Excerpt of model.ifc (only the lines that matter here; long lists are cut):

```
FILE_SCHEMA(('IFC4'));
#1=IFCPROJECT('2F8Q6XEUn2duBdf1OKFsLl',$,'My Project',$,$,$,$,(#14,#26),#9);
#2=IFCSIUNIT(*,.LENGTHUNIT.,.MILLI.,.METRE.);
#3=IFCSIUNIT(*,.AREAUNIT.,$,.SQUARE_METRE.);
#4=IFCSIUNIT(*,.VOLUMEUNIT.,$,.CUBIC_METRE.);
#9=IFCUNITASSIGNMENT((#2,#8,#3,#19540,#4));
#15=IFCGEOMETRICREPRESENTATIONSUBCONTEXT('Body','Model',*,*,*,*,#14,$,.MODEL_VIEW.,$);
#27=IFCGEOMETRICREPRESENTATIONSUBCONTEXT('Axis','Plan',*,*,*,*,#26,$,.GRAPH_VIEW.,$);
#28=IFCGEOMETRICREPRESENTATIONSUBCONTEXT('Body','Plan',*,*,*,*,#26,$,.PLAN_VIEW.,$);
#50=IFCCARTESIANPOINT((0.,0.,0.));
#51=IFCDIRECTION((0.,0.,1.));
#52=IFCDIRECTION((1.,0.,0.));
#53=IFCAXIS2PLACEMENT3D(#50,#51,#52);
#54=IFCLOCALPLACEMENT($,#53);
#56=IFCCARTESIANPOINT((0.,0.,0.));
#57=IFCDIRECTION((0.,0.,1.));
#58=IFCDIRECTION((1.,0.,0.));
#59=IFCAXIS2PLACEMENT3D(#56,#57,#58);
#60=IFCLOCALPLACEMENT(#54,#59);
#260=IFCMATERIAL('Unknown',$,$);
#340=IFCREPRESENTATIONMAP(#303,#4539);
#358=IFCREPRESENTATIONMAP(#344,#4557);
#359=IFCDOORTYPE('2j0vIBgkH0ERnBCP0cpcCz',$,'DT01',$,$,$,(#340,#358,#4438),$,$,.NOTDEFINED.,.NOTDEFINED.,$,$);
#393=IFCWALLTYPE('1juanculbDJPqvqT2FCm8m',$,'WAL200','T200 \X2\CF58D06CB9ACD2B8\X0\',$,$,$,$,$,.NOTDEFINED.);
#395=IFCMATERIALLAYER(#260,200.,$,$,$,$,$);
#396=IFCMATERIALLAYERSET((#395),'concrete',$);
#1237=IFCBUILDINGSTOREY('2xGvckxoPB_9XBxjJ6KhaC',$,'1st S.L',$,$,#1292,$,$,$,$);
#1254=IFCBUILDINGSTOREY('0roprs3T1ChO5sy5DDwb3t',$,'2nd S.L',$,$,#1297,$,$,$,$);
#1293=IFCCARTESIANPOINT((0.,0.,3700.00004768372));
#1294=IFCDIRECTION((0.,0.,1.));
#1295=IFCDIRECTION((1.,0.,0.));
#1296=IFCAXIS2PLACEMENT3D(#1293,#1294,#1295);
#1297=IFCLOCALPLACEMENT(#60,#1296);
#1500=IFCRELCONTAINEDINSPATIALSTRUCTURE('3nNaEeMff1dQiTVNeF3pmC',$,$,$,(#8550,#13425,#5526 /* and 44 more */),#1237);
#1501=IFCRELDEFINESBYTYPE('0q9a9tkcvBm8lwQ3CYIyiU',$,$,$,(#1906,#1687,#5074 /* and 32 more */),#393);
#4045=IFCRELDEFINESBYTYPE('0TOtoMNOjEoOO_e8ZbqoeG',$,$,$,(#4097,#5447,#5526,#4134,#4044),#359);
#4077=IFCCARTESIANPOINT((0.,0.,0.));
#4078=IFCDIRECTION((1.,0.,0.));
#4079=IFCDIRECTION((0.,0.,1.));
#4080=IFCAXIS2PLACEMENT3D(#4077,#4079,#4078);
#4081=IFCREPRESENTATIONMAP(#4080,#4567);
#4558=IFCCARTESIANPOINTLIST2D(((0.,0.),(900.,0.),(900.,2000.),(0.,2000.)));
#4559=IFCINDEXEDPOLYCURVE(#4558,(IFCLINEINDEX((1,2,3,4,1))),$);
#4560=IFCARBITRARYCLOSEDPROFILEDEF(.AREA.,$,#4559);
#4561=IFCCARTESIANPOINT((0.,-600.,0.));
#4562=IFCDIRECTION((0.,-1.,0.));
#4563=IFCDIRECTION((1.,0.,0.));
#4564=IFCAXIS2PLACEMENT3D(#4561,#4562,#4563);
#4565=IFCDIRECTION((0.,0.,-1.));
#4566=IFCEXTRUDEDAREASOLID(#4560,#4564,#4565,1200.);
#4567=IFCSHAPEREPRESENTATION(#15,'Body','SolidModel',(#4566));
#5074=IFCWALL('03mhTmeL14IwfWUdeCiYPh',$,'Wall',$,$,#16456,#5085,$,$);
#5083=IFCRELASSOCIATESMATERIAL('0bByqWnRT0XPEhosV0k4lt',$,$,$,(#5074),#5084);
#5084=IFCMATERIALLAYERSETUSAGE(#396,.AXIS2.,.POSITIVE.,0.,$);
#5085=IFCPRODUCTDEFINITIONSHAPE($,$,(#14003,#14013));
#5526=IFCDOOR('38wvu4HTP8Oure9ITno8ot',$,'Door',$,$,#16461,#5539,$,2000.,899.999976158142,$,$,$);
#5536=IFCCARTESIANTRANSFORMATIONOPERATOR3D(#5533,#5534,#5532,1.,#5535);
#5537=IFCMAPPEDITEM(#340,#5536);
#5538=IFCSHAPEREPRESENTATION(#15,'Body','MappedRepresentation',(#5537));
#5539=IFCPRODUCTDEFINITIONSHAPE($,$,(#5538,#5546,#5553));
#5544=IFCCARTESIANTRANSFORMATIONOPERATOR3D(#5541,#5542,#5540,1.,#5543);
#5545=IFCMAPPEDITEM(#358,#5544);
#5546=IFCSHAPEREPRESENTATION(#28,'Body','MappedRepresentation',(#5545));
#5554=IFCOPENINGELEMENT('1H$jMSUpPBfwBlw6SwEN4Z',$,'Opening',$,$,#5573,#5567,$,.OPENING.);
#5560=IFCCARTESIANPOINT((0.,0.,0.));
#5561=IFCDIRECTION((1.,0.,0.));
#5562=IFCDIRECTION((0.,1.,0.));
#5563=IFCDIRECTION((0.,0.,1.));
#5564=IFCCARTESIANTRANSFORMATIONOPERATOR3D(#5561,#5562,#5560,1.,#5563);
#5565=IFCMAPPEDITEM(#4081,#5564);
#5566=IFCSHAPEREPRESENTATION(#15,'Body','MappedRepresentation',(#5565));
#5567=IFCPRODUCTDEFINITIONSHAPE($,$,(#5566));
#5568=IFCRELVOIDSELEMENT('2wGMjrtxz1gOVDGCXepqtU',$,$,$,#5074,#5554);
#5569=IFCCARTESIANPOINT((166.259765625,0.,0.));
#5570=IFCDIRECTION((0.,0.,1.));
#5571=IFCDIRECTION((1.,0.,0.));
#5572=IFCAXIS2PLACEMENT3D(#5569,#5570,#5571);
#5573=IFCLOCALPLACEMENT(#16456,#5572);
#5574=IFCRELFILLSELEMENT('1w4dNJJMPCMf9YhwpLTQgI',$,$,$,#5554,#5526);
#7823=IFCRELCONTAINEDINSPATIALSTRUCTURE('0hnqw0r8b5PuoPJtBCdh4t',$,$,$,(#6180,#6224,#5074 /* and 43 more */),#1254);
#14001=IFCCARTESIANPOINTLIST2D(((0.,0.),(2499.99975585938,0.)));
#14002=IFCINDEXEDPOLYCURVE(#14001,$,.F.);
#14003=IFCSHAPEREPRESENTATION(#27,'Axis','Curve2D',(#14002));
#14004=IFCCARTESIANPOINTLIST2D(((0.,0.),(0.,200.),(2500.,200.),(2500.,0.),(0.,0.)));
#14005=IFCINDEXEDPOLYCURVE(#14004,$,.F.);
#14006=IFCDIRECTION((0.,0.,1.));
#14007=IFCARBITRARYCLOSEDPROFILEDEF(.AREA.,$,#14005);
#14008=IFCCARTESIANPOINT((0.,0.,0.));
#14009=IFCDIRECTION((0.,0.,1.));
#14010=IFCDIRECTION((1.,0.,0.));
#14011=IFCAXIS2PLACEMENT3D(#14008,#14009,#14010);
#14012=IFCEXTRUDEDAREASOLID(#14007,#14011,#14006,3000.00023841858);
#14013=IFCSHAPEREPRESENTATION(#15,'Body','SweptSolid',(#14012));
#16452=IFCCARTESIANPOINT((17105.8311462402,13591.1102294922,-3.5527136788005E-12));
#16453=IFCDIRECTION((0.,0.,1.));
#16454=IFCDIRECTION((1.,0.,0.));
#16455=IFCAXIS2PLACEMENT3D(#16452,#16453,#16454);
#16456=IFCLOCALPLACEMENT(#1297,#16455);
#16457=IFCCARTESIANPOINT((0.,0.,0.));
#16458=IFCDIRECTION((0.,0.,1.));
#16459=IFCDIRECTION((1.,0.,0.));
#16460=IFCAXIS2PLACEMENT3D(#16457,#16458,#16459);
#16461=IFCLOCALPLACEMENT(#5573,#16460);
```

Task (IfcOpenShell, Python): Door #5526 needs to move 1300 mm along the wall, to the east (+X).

```python
import ifcopenshell
import ifcopenshell.api.geometry
import ifcopenshell.util.placement
import ifcopenshell.util.unit

model = ifcopenshell.open("model.ifc")
unit_scale = ifcopenshell.util.unit.calculate_unit_scale(model)

door = model.by_guid("38wvu4HTP8Oure9ITno8ot")
opening = door.FillsVoids[0].RelatingOpeningElement
wall = opening.VoidsElements[0].RelatingBuildingElement

wall_matrix = ifcopenshell.util.placement.get_local_placement(wall.ObjectPlacement)
shift = wall_matrix[:3, 0] * 1.3 / unit_scale
before = ifcopenshell.util.placement.get_local_placement(door.ObjectPlacement)[:3, 3].copy()

# The door is placed relative to its opening, so it follows when the opening moves.
matrix = ifcopenshell.util.placement.get_local_placement(opening.ObjectPlacement)
matrix[:3, 3] += shift
ifcopenshell.api.geometry.edit_object_placement(
    model, product=opening, matrix=matrix, is_si=False, should_transform_children=True
)

after = ifcopenshell.util.placement.get_local_placement(door.ObjectPlacement)[:3, 3]
print("door moved by", (after - before).round(3) + 0.0)

model.write("model_edited.ifc")
```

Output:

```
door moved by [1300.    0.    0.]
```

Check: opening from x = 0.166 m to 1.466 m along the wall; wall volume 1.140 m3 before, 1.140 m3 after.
